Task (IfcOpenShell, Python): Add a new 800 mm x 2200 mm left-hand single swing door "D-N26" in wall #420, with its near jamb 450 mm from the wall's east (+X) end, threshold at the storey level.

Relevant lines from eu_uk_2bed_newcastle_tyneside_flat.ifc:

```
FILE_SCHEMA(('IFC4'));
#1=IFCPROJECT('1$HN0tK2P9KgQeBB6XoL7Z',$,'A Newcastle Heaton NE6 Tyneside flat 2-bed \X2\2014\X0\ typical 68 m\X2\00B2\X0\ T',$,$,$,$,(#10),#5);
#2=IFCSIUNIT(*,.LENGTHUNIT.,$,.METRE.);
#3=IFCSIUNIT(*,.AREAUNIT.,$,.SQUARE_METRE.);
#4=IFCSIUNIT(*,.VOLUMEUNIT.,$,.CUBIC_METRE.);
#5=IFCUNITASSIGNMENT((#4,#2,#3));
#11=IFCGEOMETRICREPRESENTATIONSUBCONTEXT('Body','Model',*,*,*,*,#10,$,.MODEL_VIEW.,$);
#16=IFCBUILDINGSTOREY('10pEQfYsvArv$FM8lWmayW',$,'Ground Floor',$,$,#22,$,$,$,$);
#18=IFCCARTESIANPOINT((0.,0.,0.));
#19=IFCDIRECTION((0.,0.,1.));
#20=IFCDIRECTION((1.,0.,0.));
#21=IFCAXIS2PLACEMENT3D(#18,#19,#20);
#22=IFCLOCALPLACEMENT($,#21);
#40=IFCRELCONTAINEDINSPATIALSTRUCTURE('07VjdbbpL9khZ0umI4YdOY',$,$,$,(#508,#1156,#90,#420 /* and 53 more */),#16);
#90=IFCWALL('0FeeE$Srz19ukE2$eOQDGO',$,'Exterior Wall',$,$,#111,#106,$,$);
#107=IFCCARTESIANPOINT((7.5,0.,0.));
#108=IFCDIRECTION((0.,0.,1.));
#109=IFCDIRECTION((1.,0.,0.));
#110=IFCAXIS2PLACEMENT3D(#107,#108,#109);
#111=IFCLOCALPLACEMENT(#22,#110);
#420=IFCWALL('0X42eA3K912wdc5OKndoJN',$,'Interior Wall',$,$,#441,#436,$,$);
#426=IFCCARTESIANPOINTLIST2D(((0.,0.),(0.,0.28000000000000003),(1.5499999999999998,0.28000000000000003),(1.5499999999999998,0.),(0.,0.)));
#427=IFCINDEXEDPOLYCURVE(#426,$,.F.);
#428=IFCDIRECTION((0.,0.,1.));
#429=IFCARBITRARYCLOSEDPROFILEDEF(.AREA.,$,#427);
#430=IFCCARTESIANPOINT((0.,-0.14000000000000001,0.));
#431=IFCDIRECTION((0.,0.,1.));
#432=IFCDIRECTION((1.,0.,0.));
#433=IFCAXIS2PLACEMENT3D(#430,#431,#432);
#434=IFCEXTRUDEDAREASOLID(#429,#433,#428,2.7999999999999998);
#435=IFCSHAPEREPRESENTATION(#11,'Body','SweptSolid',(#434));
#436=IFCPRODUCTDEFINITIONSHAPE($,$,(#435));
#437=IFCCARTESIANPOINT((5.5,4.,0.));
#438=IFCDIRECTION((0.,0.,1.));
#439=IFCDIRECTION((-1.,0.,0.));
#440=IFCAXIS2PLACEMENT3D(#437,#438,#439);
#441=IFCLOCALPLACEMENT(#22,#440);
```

```python
import numpy as np
import ifcopenshell
import ifcopenshell.api.feature
import ifcopenshell.api.geometry
import ifcopenshell.api.root
import ifcopenshell.api.spatial
import ifcopenshell.geom
import ifcopenshell.util.element
import ifcopenshell.util.placement
import ifcopenshell.util.representation
import ifcopenshell.util.shape
import ifcopenshell.util.unit

model = ifcopenshell.open("eu_uk_2bed_newcastle_tyneside_flat.ifc")
unit_scale = ifcopenshell.util.unit.calculate_unit_scale(model)
settings = ifcopenshell.geom.settings()


def volume(element):
    """Net volume in cubic metres, openings subtracted."""
    shape = ifcopenshell.geom.create_shape(settings, element)
    return ifcopenshell.util.shape.get_volume(shape.geometry)


wall = model.by_guid("0X42eA3K912wdc5OKndoJN")
storey = ifcopenshell.util.element.get_container(wall, ifc_class="IfcBuildingStorey")
context = ifcopenshell.util.representation.get_context(model, "Model", "Body", "MODEL_VIEW")
before = volume(wall)

width, height, from_end, sill = 0.8, 2.2, 0.45, 0.0  # metres

# The wall runs along its own X axis, and the end named is its -X end.
wall_shape = ifcopenshell.geom.create_shape(settings, wall)
x, y, z = ifcopenshell.util.shape.get_vertices(wall_shape.geometry).T
start = x.min() + from_end
face, thickness = float(y.min()), float(y.max() - y.min())
wall_matrix = ifcopenshell.util.placement.get_local_placement(wall.ObjectPlacement)
level = ifcopenshell.util.placement.get_local_placement(storey.ObjectPlacement)[2, 3]


def in_wall(x, y):
    """Placement at x, y metres in the wall's axes, at sill height."""
    matrix = wall_matrix.copy()
    matrix[:, 3] = wall_matrix @ np.array([x / unit_scale, y / unit_scale, 0.0, 1.0])
    matrix[2, 3] = level + sill / unit_scale
    return matrix


# Opening: a box that overshoots both wall faces by 50 mm.
opening = ifcopenshell.api.root.create_entity(model, ifc_class="IfcOpeningElement", predefined_type="OPENING")
box = ifcopenshell.api.geometry.add_wall_representation(
    model, context=context, length=width, height=height, thickness=thickness + 0.1
)
ifcopenshell.api.geometry.assign_representation(model, product=opening, representation=box)
ifcopenshell.api.geometry.edit_object_placement(model, product=opening, matrix=in_wall(start, face - 0.05), is_si=False)
ifcopenshell.api.feature.add_feature(model, feature=opening, element=wall)

door = ifcopenshell.api.root.create_entity(model, ifc_class="IfcDoor", name="D-N26", predefined_type="DOOR")
door.OverallWidth, door.OverallHeight = width / unit_scale, height / unit_scale
door.OperationType = "SINGLE_SWING_LEFT"
body = ifcopenshell.api.geometry.add_door_representation(
    model,
    context=context,
    overall_width=door.OverallWidth,
    overall_height=door.OverallHeight,
    operation_type="SINGLE_SWING_LEFT",
    lining_properties={"LiningDepth": thickness / unit_scale, "ThresholdDepth": thickness / unit_scale},
)
ifcopenshell.api.geometry.assign_representation(model, product=door, representation=body)
ifcopenshell.api.spatial.assign_container(model, products=[door], relating_structure=storey)
ifcopenshell.api.feature.add_filling(model, opening=opening, element=door)

# The lining spans the wall, so the door starts at the wall face.
ifcopenshell.api.geometry.edit_object_placement(model, product=door, matrix=in_wall(start, face), is_si=False)

after = volume(wall)

print(f"wall volume {before:.3f} -> {after:.3f} m3")

model.write("eu_uk_2bed_newcastle_tyneside_flat_v2.ifc")
```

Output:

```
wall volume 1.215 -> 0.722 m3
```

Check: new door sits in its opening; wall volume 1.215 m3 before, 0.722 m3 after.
